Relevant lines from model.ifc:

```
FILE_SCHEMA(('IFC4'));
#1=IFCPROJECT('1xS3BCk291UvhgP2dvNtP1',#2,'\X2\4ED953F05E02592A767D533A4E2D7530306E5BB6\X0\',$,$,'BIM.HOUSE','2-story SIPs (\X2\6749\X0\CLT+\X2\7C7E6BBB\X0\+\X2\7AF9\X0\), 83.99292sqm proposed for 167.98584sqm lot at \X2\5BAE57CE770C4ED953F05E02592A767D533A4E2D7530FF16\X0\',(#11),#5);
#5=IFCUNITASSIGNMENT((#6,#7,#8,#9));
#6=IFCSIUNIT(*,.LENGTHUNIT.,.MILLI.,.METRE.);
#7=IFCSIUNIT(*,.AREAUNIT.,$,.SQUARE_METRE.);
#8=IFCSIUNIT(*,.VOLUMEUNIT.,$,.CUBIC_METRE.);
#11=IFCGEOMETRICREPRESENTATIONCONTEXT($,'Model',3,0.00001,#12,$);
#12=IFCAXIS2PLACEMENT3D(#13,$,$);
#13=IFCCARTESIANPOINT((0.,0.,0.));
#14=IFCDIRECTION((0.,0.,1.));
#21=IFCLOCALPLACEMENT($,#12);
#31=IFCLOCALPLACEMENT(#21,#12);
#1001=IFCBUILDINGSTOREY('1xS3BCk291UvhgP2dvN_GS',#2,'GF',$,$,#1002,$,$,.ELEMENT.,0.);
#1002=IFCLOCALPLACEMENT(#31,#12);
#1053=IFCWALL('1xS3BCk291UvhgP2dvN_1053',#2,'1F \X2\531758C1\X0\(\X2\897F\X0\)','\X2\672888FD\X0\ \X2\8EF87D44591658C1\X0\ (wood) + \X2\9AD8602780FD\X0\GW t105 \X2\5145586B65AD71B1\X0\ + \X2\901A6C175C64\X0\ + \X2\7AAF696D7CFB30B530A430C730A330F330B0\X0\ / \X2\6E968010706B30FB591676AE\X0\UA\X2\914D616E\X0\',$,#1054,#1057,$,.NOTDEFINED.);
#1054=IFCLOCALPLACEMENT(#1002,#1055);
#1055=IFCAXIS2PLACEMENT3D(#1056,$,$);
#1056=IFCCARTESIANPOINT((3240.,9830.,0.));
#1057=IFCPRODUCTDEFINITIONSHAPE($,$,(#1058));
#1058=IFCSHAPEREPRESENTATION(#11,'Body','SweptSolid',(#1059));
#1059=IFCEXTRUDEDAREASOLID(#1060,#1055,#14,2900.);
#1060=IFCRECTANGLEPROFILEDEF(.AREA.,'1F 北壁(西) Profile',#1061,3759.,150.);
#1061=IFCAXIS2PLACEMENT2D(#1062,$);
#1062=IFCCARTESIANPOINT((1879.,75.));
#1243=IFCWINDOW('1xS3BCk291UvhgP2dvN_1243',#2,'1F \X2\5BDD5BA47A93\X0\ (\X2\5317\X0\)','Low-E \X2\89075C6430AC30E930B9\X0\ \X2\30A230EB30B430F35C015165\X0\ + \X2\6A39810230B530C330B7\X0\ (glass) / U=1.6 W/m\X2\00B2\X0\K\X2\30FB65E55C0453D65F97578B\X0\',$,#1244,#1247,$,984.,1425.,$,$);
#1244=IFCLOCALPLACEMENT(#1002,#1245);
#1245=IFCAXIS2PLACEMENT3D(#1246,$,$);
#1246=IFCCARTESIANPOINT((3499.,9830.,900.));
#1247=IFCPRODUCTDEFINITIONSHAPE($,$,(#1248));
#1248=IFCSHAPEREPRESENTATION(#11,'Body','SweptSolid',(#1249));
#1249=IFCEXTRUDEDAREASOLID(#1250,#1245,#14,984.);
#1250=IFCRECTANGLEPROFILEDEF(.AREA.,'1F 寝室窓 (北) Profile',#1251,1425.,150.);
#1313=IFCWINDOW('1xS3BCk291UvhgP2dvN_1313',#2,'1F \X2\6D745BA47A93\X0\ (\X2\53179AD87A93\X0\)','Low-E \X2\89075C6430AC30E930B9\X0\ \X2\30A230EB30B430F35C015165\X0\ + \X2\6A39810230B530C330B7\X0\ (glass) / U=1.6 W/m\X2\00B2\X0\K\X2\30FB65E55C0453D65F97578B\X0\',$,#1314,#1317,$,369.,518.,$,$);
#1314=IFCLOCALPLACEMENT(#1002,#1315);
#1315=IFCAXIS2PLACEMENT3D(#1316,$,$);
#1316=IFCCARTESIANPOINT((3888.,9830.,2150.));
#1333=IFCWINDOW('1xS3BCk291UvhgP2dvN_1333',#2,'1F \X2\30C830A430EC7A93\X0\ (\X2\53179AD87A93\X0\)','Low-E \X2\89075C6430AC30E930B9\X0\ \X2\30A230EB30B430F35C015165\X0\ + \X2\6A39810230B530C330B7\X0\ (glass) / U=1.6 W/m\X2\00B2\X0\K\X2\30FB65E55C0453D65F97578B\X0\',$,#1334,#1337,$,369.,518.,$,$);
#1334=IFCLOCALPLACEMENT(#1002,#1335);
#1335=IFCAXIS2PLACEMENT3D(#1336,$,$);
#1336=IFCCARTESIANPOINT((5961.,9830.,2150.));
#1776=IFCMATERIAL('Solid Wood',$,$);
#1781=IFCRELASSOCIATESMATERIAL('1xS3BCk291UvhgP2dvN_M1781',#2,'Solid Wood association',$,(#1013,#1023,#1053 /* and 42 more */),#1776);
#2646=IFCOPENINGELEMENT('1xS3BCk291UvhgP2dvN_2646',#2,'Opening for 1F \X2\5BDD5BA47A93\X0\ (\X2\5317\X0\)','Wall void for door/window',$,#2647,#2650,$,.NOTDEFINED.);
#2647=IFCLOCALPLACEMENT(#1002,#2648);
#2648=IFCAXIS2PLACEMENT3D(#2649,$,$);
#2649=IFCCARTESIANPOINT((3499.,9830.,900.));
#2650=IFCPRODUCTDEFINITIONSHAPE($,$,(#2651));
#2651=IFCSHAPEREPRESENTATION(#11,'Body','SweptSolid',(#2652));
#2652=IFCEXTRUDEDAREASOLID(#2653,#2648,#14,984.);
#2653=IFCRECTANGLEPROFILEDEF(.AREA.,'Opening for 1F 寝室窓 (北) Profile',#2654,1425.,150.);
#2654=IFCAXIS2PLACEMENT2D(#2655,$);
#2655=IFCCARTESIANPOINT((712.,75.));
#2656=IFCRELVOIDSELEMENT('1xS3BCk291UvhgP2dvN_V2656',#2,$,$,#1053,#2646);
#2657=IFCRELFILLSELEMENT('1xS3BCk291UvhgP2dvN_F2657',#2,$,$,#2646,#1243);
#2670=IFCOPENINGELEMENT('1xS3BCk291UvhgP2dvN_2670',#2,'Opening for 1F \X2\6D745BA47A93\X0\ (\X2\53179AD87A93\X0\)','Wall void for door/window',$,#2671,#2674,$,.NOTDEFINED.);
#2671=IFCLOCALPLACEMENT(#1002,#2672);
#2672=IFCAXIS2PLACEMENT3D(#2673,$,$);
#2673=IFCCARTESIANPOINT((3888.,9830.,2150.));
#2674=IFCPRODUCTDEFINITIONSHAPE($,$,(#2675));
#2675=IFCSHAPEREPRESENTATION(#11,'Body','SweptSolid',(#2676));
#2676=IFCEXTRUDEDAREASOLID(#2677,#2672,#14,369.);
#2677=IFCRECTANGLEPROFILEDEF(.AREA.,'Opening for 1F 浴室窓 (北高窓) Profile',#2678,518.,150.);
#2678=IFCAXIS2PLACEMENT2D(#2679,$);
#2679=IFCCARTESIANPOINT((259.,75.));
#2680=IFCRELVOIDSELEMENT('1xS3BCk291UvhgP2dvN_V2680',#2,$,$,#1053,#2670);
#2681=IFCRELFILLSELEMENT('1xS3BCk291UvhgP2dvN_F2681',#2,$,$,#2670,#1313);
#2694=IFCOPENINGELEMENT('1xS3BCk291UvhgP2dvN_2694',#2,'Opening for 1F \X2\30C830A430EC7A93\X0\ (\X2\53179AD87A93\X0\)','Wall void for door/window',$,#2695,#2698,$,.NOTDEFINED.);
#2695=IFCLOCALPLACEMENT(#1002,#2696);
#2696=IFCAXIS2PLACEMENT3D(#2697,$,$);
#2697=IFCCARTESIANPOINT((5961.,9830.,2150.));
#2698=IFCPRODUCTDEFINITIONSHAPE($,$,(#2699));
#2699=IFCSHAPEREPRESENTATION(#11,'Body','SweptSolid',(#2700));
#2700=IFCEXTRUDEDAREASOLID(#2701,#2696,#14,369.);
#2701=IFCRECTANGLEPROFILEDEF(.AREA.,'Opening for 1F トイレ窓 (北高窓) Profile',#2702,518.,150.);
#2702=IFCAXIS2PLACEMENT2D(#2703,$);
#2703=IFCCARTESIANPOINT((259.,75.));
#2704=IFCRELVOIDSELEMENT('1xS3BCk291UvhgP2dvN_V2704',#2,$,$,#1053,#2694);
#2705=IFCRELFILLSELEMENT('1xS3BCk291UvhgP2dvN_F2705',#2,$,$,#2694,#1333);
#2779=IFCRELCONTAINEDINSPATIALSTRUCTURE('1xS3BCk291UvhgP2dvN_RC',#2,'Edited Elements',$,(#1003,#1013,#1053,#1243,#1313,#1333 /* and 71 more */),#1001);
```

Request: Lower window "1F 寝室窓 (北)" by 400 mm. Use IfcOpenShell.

```python
import numpy as np
import ifcopenshell
import ifcopenshell.api.geometry
import ifcopenshell.util.placement
import ifcopenshell.util.unit

model = ifcopenshell.open("model.ifc")
unit_scale = ifcopenshell.util.unit.calculate_unit_scale(model)

window = model.by_guid("1xS3BCk291UvhgP2dvN_1243")
opening = window.FillsVoids[0].RelatingOpeningElement
dz = -0.4 / unit_scale

shift = np.array([0.0, 0.0, dz])
# The window is not placed relative to its opening, so move both.
for product in (opening, window):
    matrix = ifcopenshell.util.placement.get_local_placement(product.ObjectPlacement)
    matrix[:3, 3] += shift
    ifcopenshell.api.geometry.edit_object_placement(model, product=product, matrix=matrix, is_si=False)

print(f"moved by {dz * unit_scale:+.3f} m")

model.write("model_edited.ifc")
```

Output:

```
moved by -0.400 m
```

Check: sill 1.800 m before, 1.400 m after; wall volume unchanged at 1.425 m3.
